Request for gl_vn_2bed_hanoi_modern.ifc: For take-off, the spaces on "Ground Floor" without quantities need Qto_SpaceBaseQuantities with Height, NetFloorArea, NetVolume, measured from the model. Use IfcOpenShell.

First a look at what the model holds.

```python
import ifcopenshell
import ifcopenshell.util.element
import ifcopenshell.util.unit

model = ifcopenshell.open("gl_vn_2bed_hanoi_modern.ifc")
print(model.schema)
for unit_type in ("LENGTHUNIT", "AREAUNIT", "VOLUMEUNIT"):
    print(unit_type, ifcopenshell.util.unit.calculate_unit_scale(model, unit_type))
storey = next(s for s in model.by_type("IfcBuildingStorey") if s.Name == "Ground Floor")
spaces = [e for e in ifcopenshell.util.element.get_decomposition(storey) if e.is_a("IfcSpace")]
for e in sorted(spaces, key=lambda e: e.id()):
    print(e.id(), e.is_a(), e.Name, list(ifcopenshell.util.element.get_psets(e, qtos_only=True)), sep=" | ")
```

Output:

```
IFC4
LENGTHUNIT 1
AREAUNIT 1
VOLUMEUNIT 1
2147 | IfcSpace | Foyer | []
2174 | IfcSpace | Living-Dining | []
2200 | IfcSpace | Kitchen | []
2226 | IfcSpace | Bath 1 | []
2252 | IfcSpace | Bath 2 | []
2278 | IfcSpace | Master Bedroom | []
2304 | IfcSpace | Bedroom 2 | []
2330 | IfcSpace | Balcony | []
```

```python
import ifcopenshell
import ifcopenshell.api.pset
import ifcopenshell.geom
import ifcopenshell.util.element
import ifcopenshell.util.shape
import ifcopenshell.util.unit

model = ifcopenshell.open("gl_vn_2bed_hanoi_modern.ifc")
unit_scale = ifcopenshell.util.unit.calculate_unit_scale(model)
area_scale = ifcopenshell.util.unit.calculate_unit_scale(model, "AREAUNIT")
volume_scale = ifcopenshell.util.unit.calculate_unit_scale(model, "VOLUMEUNIT")
settings = ifcopenshell.geom.settings()

storey = next(s for s in model.by_type("IfcBuildingStorey") if s.Name == "Ground Floor")
spaces = [e for e in ifcopenshell.util.element.get_decomposition(storey) if e.is_a("IfcSpace")]

for e in sorted(spaces, key=lambda e: e.id()):
    if ifcopenshell.util.element.get_psets(e, qtos_only=True, should_inherit=False):
        continue
    # Geometry comes back in metres, in the element's own axes.
    shape = ifcopenshell.geom.create_shape(settings, e)
    values = {
        "Height": ifcopenshell.util.shape.get_z(shape.geometry) / unit_scale,
        "NetFloorArea": ifcopenshell.util.shape.get_footprint_area(shape.geometry) / area_scale,
        "NetVolume": ifcopenshell.util.shape.get_volume(shape.geometry) / volume_scale,
    }
    qto = ifcopenshell.api.pset.add_qto(model, product=e, name="Qto_SpaceBaseQuantities")
    ifcopenshell.api.pset.edit_qto(model, qto=qto, properties=values)
    print(e.id(), {k: round(v, 3) for k, v in values.items()})

model.write("gl_vn_2bed_hanoi_modern_v2.ifc")
```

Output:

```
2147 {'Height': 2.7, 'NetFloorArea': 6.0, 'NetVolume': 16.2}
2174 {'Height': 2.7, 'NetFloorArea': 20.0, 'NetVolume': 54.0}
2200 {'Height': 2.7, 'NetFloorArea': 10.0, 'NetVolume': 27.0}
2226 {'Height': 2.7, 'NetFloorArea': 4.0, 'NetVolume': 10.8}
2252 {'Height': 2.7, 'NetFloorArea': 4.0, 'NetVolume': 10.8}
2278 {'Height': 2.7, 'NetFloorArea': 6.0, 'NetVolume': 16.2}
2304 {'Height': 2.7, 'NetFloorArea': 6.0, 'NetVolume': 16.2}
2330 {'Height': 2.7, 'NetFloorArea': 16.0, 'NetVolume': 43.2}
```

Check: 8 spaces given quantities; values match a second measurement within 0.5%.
